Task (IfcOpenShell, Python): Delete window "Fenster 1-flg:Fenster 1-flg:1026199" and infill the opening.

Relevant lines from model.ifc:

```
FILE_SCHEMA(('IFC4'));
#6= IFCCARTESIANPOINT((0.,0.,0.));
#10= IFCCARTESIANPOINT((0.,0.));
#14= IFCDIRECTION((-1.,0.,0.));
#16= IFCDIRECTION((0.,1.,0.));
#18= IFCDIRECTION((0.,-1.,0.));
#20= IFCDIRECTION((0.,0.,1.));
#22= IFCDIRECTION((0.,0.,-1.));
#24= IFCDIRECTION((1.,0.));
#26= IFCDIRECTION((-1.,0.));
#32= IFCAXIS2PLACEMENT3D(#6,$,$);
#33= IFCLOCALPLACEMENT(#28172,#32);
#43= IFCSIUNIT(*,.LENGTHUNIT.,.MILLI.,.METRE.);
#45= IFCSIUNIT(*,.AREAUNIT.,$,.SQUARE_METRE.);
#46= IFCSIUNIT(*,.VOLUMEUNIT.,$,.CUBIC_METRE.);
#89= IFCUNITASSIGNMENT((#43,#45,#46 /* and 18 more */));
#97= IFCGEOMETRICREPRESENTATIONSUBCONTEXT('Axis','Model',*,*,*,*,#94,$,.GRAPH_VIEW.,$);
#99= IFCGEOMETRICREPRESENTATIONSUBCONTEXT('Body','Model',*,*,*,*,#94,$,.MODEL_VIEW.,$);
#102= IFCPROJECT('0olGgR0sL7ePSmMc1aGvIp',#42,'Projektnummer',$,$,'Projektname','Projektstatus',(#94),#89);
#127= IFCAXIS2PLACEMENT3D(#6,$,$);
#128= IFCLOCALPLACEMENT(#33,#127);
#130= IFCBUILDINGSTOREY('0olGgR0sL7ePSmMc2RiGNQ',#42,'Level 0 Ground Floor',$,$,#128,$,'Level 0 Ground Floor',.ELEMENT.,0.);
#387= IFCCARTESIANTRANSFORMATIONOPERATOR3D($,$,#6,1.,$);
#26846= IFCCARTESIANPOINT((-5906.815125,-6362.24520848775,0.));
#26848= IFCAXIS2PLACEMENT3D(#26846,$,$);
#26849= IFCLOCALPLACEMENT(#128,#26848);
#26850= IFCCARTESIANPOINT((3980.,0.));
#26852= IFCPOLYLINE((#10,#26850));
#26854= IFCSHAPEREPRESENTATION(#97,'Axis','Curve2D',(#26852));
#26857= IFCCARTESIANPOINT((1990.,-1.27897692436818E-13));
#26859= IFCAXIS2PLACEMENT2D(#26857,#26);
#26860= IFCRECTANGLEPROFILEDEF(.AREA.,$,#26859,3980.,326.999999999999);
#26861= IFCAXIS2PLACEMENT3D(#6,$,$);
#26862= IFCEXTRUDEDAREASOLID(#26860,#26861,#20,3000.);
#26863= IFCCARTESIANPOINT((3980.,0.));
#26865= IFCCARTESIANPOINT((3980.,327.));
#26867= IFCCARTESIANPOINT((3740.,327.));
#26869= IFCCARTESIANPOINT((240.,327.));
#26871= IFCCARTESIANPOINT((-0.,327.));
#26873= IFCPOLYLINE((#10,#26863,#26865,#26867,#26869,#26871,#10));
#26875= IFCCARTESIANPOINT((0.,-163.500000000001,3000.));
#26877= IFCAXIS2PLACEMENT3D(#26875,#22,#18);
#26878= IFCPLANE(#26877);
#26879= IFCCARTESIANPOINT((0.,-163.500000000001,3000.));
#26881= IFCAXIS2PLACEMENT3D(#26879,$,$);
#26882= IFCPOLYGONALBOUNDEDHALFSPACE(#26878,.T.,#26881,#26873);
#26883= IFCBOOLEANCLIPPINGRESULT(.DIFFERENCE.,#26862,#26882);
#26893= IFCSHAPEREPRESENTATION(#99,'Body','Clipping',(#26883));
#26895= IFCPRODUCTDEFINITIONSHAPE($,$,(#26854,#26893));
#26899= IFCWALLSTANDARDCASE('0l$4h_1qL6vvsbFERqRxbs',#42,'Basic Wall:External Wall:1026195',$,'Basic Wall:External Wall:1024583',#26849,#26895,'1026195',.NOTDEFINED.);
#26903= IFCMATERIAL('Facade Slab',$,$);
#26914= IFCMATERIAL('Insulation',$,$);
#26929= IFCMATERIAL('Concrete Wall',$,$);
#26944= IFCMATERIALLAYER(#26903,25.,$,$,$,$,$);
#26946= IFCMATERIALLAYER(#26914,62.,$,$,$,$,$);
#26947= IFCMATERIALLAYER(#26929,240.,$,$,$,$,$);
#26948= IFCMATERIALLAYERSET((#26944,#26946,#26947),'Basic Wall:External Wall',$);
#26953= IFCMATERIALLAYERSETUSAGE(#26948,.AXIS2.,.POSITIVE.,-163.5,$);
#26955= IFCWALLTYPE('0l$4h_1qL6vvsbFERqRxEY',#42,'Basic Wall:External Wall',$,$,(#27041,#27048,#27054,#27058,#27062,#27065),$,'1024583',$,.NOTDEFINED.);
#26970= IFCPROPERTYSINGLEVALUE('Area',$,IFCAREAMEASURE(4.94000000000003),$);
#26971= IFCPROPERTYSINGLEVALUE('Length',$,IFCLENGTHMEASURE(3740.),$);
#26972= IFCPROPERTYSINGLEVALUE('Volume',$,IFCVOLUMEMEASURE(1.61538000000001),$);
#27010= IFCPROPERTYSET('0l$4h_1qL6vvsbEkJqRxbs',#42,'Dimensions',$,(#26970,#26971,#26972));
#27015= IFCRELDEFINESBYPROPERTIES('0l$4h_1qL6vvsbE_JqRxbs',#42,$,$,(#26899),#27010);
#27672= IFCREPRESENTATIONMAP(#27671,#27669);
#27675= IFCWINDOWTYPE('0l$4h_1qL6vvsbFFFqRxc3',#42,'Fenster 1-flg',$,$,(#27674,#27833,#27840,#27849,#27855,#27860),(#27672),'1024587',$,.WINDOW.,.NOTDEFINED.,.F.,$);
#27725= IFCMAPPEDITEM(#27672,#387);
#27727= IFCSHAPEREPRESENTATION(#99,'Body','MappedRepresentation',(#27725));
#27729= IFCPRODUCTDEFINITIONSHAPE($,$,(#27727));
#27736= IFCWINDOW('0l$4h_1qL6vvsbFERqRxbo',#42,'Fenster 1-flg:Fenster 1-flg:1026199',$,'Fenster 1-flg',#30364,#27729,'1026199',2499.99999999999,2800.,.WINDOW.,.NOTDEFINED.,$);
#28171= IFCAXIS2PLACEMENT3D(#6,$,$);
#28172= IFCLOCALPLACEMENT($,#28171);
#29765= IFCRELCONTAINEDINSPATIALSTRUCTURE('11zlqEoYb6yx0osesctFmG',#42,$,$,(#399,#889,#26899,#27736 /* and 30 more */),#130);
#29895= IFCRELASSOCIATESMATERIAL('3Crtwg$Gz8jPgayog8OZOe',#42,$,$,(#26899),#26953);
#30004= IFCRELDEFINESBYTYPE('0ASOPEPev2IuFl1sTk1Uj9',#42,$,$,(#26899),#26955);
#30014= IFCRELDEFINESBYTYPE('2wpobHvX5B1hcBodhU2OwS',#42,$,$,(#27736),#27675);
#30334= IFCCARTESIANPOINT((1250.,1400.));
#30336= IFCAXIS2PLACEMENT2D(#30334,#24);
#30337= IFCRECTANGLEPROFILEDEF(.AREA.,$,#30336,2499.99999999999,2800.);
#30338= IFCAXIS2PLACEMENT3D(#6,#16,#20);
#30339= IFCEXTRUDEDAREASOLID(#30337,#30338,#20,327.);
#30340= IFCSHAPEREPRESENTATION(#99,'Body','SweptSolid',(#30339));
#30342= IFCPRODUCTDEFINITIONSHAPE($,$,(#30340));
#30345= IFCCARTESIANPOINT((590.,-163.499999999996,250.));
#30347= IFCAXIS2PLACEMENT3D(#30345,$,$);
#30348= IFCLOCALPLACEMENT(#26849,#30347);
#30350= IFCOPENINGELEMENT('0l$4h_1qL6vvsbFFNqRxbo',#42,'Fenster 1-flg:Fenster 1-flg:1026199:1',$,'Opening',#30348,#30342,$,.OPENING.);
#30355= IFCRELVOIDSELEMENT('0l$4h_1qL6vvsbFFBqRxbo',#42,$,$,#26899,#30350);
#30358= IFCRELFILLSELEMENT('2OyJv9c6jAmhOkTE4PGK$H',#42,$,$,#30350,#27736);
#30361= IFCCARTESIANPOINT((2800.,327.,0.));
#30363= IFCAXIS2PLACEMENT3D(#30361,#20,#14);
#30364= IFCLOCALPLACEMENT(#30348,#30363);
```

```python
import ifcopenshell
import ifcopenshell.api.feature
import ifcopenshell.api.pset
import ifcopenshell.api.root
import ifcopenshell.geom
import ifcopenshell.util.element
import ifcopenshell.util.shape
import ifcopenshell.util.unit

model = ifcopenshell.open("model.ifc")
area_scale = ifcopenshell.util.unit.calculate_unit_scale(model, "AREAUNIT")
volume_scale = ifcopenshell.util.unit.calculate_unit_scale(model, "VOLUMEUNIT")
settings = ifcopenshell.geom.settings()


def volume(element):
    """Net volume in cubic metres, openings subtracted."""
    shape = ifcopenshell.geom.create_shape(settings, element)
    return ifcopenshell.util.shape.get_volume(shape.geometry)


window = model.by_id(27736)
opening = window.FillsVoids[0].RelatingOpeningElement
wall = opening.VoidsElements[0].RelatingBuildingElement
before = volume(wall)

ifcopenshell.api.root.remove_product(model, product=window)
ifcopenshell.api.feature.remove_feature(model, feature=opening)

after = volume(wall)
thickness = 0.327  # wall thickness in metres

# Update the wall's stored quantities.
pset = model.by_id(ifcopenshell.util.element.get_pset(wall, "Dimensions", should_inherit=False)["id"])
ifcopenshell.api.pset.edit_pset(model, pset=pset, properties={
    "Area": model.create_entity("IfcAreaMeasure", after / thickness / area_scale),
    "Volume": model.create_entity("IfcVolumeMeasure", after / volume_scale),
})

print(f"wall volume {before:.3f} -> {after:.3f} m3")

model.write("model_updated.ifc")
```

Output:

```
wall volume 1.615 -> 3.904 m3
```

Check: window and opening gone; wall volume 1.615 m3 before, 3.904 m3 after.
